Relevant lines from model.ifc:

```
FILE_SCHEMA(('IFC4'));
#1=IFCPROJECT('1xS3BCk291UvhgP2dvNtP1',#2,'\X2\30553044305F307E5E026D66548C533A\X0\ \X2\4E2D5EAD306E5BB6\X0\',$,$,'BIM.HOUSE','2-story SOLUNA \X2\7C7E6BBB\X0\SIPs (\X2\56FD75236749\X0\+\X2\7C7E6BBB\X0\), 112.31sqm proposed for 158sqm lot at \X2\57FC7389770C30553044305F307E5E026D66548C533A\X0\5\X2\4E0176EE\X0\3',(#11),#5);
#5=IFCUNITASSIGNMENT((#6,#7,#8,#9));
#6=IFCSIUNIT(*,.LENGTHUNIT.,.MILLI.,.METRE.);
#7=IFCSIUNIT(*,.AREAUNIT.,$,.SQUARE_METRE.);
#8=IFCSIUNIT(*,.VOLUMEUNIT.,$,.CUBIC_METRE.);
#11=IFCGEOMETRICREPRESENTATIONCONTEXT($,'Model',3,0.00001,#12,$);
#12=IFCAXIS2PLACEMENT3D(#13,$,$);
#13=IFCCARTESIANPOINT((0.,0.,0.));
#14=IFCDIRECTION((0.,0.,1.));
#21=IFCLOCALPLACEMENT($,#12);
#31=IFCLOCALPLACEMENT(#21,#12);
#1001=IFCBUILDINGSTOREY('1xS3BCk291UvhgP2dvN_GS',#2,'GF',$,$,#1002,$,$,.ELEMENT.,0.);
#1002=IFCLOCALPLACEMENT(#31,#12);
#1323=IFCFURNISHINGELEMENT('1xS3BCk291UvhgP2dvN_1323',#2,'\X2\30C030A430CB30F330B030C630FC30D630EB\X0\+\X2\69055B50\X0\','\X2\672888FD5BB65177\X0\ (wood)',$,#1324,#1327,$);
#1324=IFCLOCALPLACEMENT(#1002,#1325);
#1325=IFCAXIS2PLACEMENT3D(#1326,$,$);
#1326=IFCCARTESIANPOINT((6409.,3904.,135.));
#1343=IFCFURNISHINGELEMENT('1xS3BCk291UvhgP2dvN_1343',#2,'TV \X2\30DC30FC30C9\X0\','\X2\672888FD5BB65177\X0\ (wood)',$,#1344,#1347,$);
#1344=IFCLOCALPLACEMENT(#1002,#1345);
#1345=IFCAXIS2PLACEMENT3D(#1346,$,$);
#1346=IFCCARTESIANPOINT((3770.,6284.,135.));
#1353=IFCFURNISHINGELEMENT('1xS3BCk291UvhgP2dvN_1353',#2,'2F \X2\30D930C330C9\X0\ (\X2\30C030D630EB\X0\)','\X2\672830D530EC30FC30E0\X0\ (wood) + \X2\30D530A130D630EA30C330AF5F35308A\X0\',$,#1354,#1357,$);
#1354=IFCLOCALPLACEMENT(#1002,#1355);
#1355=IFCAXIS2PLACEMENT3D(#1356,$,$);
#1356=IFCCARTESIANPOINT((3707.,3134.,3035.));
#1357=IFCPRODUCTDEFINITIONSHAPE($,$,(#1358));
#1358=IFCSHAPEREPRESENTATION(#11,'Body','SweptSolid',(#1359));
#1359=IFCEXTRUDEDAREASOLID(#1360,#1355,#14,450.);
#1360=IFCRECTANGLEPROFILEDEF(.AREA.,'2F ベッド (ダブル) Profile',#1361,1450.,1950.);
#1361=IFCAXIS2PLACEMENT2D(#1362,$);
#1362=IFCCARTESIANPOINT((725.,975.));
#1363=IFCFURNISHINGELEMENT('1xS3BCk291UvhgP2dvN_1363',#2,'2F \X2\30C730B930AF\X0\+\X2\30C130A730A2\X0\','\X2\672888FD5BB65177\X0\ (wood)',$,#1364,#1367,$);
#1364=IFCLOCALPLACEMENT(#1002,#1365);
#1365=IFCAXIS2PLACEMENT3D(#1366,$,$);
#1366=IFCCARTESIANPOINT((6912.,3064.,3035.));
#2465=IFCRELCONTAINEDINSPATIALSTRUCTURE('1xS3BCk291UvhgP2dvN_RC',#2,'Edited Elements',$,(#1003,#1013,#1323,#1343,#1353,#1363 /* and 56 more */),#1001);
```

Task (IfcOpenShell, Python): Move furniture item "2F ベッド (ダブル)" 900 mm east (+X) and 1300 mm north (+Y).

```python
import ifcopenshell
import ifcopenshell.api.geometry
import ifcopenshell.util.placement
import ifcopenshell.util.unit

model = ifcopenshell.open("model.ifc")
unit_scale = ifcopenshell.util.unit.calculate_unit_scale(model)

item = model.by_guid("1xS3BCk291UvhgP2dvN_1353")
matrix = ifcopenshell.util.placement.get_local_placement(item.ObjectPlacement)
matrix[0, 3] += 0.9 / unit_scale
matrix[1, 3] += 1.3 / unit_scale
ifcopenshell.api.geometry.edit_object_placement(model, product=item, matrix=matrix, is_si=False)

print(ifcopenshell.util.placement.get_local_placement(item.ObjectPlacement).round(3) + 0.0)

model.write("model_rev.ifc")
```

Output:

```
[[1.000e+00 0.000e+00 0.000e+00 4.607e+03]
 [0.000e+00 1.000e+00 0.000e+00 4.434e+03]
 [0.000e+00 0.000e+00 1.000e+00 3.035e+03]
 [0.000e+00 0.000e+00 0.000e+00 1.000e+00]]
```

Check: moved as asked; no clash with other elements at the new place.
